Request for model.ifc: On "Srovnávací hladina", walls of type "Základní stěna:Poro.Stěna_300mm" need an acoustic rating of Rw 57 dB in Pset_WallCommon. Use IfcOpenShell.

First a look at what the model holds.

```python
import ifcopenshell
import ifcopenshell.util.element

model = ifcopenshell.open("model.ifc")
print(model.schema)
storey = next(s for s in model.by_type("IfcBuildingStorey") if s.Name == "Srovnávací hladina")
walls = [e for e in ifcopenshell.util.element.get_decomposition(storey) if e.is_a("IfcWall")]
seen = {}
for e in walls:
    element_type = ifcopenshell.util.element.get_type(e)
    key = (element_type.Name if element_type != e and element_type else None, ifcopenshell.util.element.get_pset(e, "Pset_WallCommon", "AcousticRating"))
    seen[key] = seen.get(key, 0) + 1
for (name, value), count in sorted(seen.items(), key=str):
    print(count, "x", name, "|", value)
```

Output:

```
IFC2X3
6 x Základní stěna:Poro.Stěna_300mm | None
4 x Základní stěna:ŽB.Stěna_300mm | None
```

```python
import ifcopenshell
import ifcopenshell.api.pset
import ifcopenshell.util.element

model = ifcopenshell.open("model.ifc")

storey = next(s for s in model.by_type("IfcBuildingStorey") if s.Name == "Srovnávací hladina")
walls = [e for e in ifcopenshell.util.element.get_decomposition(storey) if e.is_a("IfcWall")]

count = 0
for e in walls:
    element_type = ifcopenshell.util.element.get_type(e)
    if element_type in (None, e) or element_type.Name != "Základní stěna:Poro.Stěna_300mm":
        continue
    # add_pset returns the element's existing set when there is one.
    pset = ifcopenshell.api.pset.add_pset(model, product=e, name="Pset_WallCommon")
    ifcopenshell.api.pset.edit_pset(model, pset=pset, properties={"AcousticRating": "Rw 57 dB"})
    count += 1

print(count, "walls updated")

model.write("model_edited.ifc")
```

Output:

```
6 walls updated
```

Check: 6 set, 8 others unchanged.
